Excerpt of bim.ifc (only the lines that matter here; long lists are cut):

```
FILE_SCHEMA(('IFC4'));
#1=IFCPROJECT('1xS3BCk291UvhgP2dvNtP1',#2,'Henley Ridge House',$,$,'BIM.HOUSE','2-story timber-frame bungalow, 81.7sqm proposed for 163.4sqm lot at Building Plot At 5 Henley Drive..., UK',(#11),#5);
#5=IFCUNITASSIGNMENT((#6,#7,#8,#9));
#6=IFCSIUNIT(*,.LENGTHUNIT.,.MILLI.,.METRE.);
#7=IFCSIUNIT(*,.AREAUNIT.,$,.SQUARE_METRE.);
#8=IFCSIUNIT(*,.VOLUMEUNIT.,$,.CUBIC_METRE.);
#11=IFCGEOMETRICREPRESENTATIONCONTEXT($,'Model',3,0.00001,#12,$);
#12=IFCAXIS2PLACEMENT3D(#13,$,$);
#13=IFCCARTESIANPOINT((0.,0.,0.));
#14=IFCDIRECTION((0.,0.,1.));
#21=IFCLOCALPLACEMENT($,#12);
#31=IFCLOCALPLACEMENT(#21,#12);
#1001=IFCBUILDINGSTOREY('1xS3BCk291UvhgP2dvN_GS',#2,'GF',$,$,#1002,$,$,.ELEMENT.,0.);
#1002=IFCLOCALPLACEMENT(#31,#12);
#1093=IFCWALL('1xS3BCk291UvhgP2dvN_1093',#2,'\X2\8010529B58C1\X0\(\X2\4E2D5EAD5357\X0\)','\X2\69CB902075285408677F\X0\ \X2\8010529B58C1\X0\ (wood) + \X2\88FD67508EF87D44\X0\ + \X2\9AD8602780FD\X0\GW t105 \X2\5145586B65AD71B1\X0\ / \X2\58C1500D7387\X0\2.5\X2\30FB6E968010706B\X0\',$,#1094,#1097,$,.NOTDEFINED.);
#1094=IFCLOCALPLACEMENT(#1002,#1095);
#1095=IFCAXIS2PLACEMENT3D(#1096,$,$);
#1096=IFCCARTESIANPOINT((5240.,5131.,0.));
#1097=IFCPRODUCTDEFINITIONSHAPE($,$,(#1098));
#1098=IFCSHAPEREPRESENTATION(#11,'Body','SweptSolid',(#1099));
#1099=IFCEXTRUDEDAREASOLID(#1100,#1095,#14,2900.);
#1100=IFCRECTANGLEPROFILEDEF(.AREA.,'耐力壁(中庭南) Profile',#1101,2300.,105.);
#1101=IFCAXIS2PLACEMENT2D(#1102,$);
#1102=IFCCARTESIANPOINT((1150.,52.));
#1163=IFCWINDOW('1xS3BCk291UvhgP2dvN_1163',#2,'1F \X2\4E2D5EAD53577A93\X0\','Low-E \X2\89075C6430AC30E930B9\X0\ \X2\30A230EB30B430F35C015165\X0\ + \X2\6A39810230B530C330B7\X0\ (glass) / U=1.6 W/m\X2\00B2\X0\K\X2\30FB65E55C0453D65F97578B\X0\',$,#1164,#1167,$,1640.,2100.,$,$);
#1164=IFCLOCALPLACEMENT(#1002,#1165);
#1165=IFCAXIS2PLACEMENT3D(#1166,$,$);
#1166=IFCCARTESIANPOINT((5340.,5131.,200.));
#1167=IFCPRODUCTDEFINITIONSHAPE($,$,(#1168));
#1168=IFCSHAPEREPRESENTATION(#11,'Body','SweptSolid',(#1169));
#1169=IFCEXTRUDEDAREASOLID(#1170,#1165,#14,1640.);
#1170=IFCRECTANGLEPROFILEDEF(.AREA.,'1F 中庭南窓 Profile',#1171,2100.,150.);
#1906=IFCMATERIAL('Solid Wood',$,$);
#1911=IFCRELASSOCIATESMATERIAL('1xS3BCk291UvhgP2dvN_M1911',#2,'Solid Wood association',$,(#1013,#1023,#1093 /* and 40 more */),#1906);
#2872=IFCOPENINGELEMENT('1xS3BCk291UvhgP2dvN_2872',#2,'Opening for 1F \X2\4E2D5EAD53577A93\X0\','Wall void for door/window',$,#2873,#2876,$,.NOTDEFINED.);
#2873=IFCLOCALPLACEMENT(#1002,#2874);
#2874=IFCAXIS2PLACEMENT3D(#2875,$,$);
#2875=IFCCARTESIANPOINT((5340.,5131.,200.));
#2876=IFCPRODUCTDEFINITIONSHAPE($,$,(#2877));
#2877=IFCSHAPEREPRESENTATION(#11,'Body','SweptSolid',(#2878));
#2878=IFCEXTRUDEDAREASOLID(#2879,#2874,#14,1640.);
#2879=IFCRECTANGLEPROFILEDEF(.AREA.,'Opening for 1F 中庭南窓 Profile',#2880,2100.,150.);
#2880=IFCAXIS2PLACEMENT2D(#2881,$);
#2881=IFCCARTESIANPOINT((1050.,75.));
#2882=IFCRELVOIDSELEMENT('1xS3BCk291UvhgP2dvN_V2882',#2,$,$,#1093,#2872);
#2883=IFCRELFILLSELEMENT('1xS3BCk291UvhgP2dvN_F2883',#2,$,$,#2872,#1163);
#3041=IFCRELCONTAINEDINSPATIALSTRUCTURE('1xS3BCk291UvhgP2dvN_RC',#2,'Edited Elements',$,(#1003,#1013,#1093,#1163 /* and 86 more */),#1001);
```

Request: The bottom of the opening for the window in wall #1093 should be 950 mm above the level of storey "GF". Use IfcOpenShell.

```python
import numpy as np
import ifcopenshell
import ifcopenshell.api.geometry
import ifcopenshell.geom
import ifcopenshell.util.element
import ifcopenshell.util.placement
import ifcopenshell.util.shape
import ifcopenshell.util.unit

model = ifcopenshell.open("bim.ifc")
unit_scale = ifcopenshell.util.unit.calculate_unit_scale(model)

window = model.by_guid("1xS3BCk291UvhgP2dvN_1163")
opening = window.FillsVoids[0].RelatingOpeningElement
storey = ifcopenshell.util.element.get_container(window, ifc_class="IfcBuildingStorey")
level = ifcopenshell.util.placement.get_local_placement(storey.ObjectPlacement)[2, 3]

# The opening's origin need not be at the sill, so measure its lowest point.
shape = ifcopenshell.geom.create_shape(ifcopenshell.geom.settings(), opening)
bottom = ifcopenshell.util.shape.get_shape_bottom_elevation(shape, shape.geometry) / unit_scale
dz = level + 0.95 / unit_scale - bottom

shift = np.array([0.0, 0.0, dz])
# The window is not placed relative to its opening, so move both.
for product in (opening, window):
    matrix = ifcopenshell.util.placement.get_local_placement(product.ObjectPlacement)
    matrix[:3, 3] += shift
    ifcopenshell.api.geometry.edit_object_placement(model, product=product, matrix=matrix, is_si=False)

print(f"moved by {dz * unit_scale:+.3f} m")

model.write("bim_v2.ifc")
```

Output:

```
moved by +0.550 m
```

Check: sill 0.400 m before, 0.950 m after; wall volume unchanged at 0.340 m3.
